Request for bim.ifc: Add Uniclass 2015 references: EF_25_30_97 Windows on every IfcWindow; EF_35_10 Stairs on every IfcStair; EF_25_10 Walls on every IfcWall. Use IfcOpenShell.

First a look at what the model holds.

```python
import ifcopenshell

model = ifcopenshell.open("bim.ifc")
print(model.schema)
print("classifications:", [c.Name for c in model.by_type("IfcClassification")])
for ifc_class in ("IfcDoor", "IfcRoof", "IfcStair", "IfcWall", "IfcWindow"):
    print(ifc_class, len(model.by_type(ifc_class)))
```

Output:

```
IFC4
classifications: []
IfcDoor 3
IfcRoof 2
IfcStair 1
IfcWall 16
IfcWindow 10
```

```python
import ifcopenshell
import ifcopenshell.api.classification

model = ifcopenshell.open("bim.ifc")

system = ifcopenshell.api.classification.add_classification(model, classification="Uniclass 2015")

codes = {
    "IfcWindow": ("EF_25_30_97", "Windows"),
    "IfcStair": ("EF_35_10", "Stairs"),
    "IfcWall": ("EF_25_10", "Walls"),
}
for ifc_class, (code, name) in codes.items():
    products = model.by_type(ifc_class)
    ifcopenshell.api.classification.add_reference(
        model, products=products, classification=system, identification=code, name=name
    )
    print(code, len(products))

model.write("bim_v2.ifc")
```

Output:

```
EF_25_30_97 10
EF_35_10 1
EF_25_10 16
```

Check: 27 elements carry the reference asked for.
